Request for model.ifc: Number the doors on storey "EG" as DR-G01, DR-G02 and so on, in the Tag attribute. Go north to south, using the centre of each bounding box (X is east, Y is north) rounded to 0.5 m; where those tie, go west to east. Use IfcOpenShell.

First a look at what the model holds.

```python
import ifcopenshell
import ifcopenshell.util.element
import ifcopenshell.util.placement

model = ifcopenshell.open("model.ifc")
print(model.schema)
storey = next(s for s in model.by_type("IfcBuildingStorey") if s.Name == "EG")
doors = [e for e in ifcopenshell.util.element.get_decomposition(storey) if e.is_a("IfcDoor")]
for e in sorted(doors, key=lambda e: e.id()):
    origin = ifcopenshell.util.placement.get_local_placement(e.ObjectPlacement)[:3, 3]
    print(e.id(), e.Tag, e.Name, origin.round(2) + 0.0, sep=" | ")
```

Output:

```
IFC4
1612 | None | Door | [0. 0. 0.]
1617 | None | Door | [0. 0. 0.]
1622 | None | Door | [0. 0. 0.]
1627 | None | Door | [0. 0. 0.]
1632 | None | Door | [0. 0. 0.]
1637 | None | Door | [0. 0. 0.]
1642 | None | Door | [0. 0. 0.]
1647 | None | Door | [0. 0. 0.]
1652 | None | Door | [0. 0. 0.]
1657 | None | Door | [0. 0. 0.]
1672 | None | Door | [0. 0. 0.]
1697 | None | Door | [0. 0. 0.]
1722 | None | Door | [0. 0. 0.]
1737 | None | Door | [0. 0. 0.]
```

```python
import ifcopenshell
import ifcopenshell.geom
import ifcopenshell.util.element
import ifcopenshell.util.shape

model = ifcopenshell.open("model.ifc")
settings = ifcopenshell.geom.settings()
settings.set("use-world-coords", True)


def centre(element):
    shape = ifcopenshell.geom.create_shape(settings, element)
    return ifcopenshell.util.shape.get_bbox_centroid(shape.geometry)


storey = next(s for s in model.by_type("IfcBuildingStorey") if s.Name == "EG")
doors = [e for e in ifcopenshell.util.element.get_decomposition(storey) if e.is_a("IfcDoor")]

# Insertion points can sit at a corner or the storey origin, so sort by the geometry (in metres).
centres = {e: centre(e) for e in doors}
doors.sort(key=lambda e: (-round(centres[e][1] / 0.5), centres[e][0]))

for i, e in enumerate(doors, start=1):
    number = f"DR-G{i:02d}"
    e.Tag = number
    print(e.id(), number)

model.write("model-out.ifc")
```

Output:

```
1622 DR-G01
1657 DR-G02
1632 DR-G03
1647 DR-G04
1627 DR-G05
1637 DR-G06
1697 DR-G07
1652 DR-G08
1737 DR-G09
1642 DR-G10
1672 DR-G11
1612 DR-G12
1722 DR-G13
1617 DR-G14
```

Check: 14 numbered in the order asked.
